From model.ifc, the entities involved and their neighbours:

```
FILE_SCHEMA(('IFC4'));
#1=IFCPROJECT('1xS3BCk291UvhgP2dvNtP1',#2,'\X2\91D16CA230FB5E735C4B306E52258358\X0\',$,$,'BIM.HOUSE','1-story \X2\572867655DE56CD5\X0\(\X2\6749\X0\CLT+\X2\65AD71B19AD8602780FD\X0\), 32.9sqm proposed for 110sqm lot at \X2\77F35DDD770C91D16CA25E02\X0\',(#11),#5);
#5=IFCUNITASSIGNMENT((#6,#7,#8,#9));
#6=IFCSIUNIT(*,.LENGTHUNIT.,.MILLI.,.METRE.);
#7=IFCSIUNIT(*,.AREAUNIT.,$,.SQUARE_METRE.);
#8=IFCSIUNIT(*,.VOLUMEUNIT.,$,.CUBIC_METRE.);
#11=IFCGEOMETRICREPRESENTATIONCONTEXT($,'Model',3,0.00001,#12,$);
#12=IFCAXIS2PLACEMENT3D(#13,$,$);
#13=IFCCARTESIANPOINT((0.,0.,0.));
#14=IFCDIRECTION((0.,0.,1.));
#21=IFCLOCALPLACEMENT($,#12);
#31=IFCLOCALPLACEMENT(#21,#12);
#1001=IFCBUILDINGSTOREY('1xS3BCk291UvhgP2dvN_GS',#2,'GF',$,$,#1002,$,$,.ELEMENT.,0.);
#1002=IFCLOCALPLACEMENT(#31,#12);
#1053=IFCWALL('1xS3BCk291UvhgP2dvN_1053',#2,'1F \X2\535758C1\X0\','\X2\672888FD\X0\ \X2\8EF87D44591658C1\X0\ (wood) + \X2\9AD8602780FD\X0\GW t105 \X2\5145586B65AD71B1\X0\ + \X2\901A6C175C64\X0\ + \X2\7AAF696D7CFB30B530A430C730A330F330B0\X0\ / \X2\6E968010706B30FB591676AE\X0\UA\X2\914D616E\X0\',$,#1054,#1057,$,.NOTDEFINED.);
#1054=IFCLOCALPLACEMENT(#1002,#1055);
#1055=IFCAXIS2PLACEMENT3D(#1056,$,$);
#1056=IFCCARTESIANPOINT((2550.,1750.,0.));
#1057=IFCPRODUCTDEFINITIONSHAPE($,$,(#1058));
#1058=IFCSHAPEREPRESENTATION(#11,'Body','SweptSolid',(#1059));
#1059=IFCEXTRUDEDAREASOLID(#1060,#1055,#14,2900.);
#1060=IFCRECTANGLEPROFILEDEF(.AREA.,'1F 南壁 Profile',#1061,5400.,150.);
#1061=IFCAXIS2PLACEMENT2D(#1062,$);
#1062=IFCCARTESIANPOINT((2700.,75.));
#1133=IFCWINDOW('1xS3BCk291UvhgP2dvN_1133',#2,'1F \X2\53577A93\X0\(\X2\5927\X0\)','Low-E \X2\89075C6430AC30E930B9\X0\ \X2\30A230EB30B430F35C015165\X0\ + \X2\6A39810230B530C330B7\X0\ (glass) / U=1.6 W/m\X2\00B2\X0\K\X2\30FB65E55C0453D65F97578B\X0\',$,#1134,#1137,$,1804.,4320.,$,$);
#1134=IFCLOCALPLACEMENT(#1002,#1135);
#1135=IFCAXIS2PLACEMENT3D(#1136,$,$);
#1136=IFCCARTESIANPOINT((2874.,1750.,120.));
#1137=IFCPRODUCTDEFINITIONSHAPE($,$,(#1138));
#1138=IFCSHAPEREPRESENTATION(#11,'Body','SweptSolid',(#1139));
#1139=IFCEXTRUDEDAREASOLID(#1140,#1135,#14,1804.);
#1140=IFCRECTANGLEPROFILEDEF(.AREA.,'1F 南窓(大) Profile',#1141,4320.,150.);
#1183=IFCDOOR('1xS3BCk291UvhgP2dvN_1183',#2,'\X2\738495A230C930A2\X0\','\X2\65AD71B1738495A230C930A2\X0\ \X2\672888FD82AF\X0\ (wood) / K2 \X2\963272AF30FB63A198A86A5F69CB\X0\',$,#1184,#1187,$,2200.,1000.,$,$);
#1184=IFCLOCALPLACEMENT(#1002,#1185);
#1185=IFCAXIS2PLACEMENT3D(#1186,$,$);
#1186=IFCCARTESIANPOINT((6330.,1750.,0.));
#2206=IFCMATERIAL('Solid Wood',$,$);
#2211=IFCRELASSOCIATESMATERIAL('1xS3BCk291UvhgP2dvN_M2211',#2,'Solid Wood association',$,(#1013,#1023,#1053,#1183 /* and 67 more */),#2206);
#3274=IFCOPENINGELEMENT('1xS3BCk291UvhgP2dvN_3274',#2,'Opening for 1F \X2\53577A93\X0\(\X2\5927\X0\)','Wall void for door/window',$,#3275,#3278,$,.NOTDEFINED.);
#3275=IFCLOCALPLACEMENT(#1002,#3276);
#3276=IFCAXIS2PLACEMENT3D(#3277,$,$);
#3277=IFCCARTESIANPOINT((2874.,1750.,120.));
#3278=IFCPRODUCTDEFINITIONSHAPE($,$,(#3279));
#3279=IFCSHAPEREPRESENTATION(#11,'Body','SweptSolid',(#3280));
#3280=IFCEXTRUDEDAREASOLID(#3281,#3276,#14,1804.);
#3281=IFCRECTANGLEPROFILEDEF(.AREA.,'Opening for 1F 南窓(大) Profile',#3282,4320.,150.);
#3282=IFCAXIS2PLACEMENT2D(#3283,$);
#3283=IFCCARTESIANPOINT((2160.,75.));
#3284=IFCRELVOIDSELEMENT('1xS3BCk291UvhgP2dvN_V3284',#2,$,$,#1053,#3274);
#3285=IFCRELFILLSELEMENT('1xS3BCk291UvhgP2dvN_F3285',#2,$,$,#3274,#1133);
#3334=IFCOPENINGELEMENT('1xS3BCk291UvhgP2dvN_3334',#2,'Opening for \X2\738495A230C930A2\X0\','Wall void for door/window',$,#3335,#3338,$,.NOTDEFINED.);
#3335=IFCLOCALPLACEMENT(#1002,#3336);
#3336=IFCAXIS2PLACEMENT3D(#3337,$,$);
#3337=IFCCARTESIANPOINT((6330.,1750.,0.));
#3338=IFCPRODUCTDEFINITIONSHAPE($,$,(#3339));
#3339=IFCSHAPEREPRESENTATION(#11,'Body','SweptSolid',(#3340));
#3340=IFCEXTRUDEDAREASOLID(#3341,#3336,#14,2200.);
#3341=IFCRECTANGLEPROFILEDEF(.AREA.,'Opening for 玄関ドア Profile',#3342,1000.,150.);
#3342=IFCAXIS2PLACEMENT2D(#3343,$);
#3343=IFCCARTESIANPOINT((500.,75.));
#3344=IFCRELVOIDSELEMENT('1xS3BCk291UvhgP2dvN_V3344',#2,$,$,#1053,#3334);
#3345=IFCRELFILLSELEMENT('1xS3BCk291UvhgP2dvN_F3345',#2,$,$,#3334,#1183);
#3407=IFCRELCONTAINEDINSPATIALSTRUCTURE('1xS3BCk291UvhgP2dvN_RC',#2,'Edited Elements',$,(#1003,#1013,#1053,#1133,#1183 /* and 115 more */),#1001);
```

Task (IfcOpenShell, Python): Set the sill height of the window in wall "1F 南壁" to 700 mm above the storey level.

```python
import numpy as np
import ifcopenshell
import ifcopenshell.api.geometry
import ifcopenshell.geom
import ifcopenshell.util.element
import ifcopenshell.util.placement
import ifcopenshell.util.shape
import ifcopenshell.util.unit

model = ifcopenshell.open("model.ifc")
unit_scale = ifcopenshell.util.unit.calculate_unit_scale(model)

window = model.by_guid("1xS3BCk291UvhgP2dvN_1133")
opening = window.FillsVoids[0].RelatingOpeningElement
storey = ifcopenshell.util.element.get_container(window, ifc_class="IfcBuildingStorey")
level = ifcopenshell.util.placement.get_local_placement(storey.ObjectPlacement)[2, 3]

# The opening's origin need not be at the sill, so measure its lowest point.
shape = ifcopenshell.geom.create_shape(ifcopenshell.geom.settings(), opening)
bottom = ifcopenshell.util.shape.get_shape_bottom_elevation(shape, shape.geometry) / unit_scale
dz = level + 700.0 - bottom

shift = np.array([0.0, 0.0, dz])
# The window is not placed relative to its opening, so move both.
for product in (opening, window):
    matrix = ifcopenshell.util.placement.get_local_placement(product.ObjectPlacement)
    matrix[:3, 3] += shift
    ifcopenshell.api.geometry.edit_object_placement(model, product=product, matrix=matrix, is_si=False)

print(f"moved by {dz * unit_scale:+.3f} m")

model.write("model-out.ifc")
```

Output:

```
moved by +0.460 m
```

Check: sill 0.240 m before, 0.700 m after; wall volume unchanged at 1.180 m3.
